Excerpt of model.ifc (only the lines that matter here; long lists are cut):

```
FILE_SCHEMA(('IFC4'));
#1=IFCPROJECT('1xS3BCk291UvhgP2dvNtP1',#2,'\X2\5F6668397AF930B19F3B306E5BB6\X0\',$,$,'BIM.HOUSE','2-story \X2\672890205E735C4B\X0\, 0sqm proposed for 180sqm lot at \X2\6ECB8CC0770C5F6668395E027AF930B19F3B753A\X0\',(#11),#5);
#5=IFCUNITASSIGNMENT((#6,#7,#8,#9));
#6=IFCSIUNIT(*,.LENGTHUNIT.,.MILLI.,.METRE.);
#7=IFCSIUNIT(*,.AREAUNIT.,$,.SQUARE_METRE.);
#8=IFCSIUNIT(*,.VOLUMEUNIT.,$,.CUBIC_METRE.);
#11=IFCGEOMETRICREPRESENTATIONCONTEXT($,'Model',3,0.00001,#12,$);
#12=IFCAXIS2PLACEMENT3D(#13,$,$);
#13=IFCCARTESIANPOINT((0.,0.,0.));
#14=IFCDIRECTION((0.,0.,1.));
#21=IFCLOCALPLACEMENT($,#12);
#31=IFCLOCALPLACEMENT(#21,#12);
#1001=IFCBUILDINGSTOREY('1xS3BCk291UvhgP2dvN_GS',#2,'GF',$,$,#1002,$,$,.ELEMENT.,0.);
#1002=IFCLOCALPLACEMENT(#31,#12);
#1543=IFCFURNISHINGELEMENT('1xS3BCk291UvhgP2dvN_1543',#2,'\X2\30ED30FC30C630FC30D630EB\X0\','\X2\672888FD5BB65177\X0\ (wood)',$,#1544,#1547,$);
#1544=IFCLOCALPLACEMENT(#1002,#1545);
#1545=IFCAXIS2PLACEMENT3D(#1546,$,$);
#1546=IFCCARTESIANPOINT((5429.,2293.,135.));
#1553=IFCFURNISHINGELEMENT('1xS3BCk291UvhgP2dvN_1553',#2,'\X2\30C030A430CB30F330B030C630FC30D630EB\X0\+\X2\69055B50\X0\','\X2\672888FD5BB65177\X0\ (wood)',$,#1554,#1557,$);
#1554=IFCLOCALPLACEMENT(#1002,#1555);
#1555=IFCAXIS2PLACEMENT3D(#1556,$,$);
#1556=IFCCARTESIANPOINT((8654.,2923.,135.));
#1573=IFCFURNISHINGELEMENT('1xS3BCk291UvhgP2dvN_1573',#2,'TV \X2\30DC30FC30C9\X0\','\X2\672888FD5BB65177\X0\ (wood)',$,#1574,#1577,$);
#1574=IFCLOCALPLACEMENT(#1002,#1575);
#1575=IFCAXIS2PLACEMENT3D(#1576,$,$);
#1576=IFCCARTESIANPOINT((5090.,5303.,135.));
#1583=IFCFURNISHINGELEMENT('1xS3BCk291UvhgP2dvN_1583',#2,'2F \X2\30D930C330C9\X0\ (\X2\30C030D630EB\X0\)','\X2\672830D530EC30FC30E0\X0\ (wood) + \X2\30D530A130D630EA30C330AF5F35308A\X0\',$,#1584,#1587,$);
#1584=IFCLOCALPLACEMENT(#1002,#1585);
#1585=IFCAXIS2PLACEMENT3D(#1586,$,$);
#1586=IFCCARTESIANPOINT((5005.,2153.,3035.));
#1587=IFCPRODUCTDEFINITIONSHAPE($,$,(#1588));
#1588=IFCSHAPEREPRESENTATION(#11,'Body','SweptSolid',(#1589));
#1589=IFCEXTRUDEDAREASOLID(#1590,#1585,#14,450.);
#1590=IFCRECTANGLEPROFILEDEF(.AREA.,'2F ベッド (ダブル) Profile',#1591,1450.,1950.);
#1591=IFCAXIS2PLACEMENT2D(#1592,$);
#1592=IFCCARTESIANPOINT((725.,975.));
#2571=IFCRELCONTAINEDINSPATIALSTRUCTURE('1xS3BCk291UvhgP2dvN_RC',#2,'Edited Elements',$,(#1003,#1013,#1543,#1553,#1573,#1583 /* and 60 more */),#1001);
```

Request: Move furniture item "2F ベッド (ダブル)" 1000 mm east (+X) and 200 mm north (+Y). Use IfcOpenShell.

```python
import ifcopenshell
import ifcopenshell.api.geometry
import ifcopenshell.util.placement
import ifcopenshell.util.unit

model = ifcopenshell.open("model.ifc")
unit_scale = ifcopenshell.util.unit.calculate_unit_scale(model)

item = model.by_id(1583)
matrix = ifcopenshell.util.placement.get_local_placement(item.ObjectPlacement)
matrix[0, 3] += 1 / unit_scale
matrix[1, 3] += 0.2 / unit_scale
ifcopenshell.api.geometry.edit_object_placement(model, product=item, matrix=matrix, is_si=False)

print(ifcopenshell.util.placement.get_local_placement(item.ObjectPlacement).round(3) + 0.0)

model.write("model_updated.ifc")
```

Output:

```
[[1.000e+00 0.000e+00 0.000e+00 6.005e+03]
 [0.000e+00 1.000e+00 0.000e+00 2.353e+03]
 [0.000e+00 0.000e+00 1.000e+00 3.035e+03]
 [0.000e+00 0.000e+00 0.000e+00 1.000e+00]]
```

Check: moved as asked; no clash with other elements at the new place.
